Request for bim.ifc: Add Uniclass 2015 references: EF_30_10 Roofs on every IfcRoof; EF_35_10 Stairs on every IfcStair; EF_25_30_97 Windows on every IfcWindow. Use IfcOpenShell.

First a look at what the model holds.

```python
import ifcopenshell

model = ifcopenshell.open("bim.ifc")
print(model.schema)
print("classifications:", [c.Name for c in model.by_type("IfcClassification")])
for ifc_class in ("IfcDoor", "IfcRoof", "IfcStair", "IfcWall", "IfcWindow"):
    print(ifc_class, len(model.by_type(ifc_class)))
```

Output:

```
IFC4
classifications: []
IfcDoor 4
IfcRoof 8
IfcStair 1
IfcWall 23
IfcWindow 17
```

```python
import ifcopenshell
import ifcopenshell.api.classification

model = ifcopenshell.open("bim.ifc")

system = ifcopenshell.api.classification.add_classification(model, classification="Uniclass 2015")

codes = {
    "IfcRoof": ("EF_30_10", "Roofs"),
    "IfcStair": ("EF_35_10", "Stairs"),
    "IfcWindow": ("EF_25_30_97", "Windows"),
}
for ifc_class, (code, name) in codes.items():
    products = model.by_type(ifc_class)
    ifcopenshell.api.classification.add_reference(
        model, products=products, classification=system, identification=code, name=name
    )
    print(code, len(products))

model.write("bim_edited.ifc")
```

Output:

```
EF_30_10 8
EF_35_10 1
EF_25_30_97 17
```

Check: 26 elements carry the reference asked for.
